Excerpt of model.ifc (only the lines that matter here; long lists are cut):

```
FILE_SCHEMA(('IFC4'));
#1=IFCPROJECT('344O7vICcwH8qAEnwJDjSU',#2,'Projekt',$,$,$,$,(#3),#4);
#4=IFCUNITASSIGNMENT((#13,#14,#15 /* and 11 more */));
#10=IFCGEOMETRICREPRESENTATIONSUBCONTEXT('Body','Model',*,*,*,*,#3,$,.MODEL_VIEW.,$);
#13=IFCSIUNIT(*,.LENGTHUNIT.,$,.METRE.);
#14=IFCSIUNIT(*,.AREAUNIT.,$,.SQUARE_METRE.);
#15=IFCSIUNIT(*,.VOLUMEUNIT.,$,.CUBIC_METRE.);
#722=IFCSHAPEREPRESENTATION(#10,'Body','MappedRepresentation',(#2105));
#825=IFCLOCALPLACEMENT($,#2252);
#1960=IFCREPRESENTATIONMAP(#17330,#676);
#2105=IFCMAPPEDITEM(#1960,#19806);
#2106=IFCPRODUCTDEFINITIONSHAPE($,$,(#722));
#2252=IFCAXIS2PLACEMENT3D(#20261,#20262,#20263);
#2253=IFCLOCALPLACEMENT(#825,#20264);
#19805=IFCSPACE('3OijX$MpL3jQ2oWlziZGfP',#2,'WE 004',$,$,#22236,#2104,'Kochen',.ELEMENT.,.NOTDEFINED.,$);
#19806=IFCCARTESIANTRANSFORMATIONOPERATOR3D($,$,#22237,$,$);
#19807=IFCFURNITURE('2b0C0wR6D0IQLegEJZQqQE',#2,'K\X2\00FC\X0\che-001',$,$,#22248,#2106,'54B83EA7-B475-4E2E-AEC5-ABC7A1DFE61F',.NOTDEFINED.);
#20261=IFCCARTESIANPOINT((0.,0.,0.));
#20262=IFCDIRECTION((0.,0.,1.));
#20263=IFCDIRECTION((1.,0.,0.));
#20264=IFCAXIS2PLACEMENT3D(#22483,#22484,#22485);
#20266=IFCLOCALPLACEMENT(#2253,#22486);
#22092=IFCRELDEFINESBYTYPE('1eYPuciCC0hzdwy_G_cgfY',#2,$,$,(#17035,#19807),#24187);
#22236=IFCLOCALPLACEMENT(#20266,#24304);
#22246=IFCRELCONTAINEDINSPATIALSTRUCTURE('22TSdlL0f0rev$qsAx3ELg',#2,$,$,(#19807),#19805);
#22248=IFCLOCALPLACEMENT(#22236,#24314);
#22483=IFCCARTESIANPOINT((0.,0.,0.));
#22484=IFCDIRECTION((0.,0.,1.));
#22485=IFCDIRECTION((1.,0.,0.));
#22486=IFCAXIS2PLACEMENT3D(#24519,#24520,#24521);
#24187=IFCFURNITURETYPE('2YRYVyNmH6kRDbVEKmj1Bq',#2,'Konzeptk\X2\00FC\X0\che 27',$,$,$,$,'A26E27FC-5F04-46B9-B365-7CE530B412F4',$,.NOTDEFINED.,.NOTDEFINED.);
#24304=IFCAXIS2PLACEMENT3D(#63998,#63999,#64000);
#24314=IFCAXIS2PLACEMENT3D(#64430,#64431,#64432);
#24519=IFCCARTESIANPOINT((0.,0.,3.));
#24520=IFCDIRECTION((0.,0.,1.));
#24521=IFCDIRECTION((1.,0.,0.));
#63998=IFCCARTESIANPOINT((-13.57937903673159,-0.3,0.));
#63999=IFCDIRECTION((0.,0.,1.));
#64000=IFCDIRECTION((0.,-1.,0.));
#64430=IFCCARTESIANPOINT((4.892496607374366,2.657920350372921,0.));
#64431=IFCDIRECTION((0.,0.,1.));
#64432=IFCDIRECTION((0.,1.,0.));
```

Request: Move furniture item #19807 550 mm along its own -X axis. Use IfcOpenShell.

```python
import ifcopenshell
import ifcopenshell.api.geometry
import ifcopenshell.util.placement
import ifcopenshell.util.unit

model = ifcopenshell.open("model.ifc")
unit_scale = ifcopenshell.util.unit.calculate_unit_scale(model)

item = model.by_guid("2b0C0wR6D0IQLegEJZQqQE")
matrix = ifcopenshell.util.placement.get_local_placement(item.ObjectPlacement)
matrix[:3, 3] -= matrix[:3, 0] * 0.55 / unit_scale
ifcopenshell.api.geometry.edit_object_placement(model, product=item, matrix=matrix, is_si=False)

print(ifcopenshell.util.placement.get_local_placement(item.ObjectPlacement).round(3) + 0.0)

model.write("model_updated.ifc")
```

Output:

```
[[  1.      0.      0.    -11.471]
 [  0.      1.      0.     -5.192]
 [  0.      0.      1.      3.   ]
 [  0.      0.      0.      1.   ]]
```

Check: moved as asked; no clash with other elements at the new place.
